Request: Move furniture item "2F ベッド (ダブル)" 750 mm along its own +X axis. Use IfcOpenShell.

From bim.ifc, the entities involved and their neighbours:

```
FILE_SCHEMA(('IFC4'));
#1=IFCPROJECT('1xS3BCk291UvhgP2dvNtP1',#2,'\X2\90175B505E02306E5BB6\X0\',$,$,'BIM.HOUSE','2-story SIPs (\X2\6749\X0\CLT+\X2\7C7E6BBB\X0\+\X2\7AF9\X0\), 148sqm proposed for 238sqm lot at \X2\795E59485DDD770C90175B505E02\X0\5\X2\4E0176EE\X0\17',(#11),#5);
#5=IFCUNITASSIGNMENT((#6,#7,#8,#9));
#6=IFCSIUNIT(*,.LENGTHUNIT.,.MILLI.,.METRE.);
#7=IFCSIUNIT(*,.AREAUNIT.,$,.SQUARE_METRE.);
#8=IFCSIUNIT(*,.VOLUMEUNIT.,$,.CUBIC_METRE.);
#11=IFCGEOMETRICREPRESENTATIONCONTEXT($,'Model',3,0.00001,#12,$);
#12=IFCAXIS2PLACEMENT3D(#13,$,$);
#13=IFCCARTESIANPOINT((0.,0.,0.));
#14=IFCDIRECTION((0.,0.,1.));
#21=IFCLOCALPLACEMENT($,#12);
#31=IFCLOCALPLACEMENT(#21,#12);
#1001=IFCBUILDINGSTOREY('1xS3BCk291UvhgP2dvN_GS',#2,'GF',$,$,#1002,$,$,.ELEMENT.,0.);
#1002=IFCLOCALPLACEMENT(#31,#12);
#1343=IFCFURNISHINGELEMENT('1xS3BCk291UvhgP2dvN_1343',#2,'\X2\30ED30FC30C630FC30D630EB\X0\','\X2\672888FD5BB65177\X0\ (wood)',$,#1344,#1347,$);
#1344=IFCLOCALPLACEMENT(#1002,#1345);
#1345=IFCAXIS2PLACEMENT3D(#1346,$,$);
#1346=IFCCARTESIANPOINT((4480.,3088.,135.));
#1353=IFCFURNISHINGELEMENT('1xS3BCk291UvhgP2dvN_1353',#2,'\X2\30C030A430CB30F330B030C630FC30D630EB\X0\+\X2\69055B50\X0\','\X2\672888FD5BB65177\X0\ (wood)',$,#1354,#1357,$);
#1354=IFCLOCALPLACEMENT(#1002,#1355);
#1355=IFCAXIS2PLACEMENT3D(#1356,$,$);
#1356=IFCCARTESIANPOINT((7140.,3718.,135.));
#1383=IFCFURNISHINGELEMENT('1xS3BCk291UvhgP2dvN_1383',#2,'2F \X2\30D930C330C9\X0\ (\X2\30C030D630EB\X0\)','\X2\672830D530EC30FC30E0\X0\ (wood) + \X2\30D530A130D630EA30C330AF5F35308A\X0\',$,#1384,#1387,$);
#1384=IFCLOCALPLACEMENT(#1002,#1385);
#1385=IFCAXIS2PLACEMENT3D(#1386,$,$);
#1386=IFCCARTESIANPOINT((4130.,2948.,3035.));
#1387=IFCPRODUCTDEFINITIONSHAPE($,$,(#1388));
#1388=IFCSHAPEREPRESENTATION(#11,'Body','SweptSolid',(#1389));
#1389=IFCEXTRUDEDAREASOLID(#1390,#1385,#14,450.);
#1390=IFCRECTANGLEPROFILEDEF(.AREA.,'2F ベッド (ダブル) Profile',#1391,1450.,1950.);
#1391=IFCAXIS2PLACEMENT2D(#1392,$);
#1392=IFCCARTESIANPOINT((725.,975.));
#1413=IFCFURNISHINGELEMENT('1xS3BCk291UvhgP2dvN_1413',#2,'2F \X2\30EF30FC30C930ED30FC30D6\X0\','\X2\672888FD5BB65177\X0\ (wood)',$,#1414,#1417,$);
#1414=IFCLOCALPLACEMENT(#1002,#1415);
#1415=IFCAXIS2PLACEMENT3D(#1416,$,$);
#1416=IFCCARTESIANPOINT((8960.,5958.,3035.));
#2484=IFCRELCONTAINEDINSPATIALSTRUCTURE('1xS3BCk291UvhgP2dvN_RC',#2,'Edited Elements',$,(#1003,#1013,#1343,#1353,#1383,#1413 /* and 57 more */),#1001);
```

```python
import ifcopenshell
import ifcopenshell.api.geometry
import ifcopenshell.util.placement
import ifcopenshell.util.unit

model = ifcopenshell.open("bim.ifc")
unit_scale = ifcopenshell.util.unit.calculate_unit_scale(model)

item = model.by_guid("1xS3BCk291UvhgP2dvN_1383")
matrix = ifcopenshell.util.placement.get_local_placement(item.ObjectPlacement)
matrix[:3, 3] += matrix[:3, 0] * 0.75 / unit_scale
ifcopenshell.api.geometry.edit_object_placement(model, product=item, matrix=matrix, is_si=False)

print(ifcopenshell.util.placement.get_local_placement(item.ObjectPlacement).round(3) + 0.0)

model.write("bim_rev.ifc")
```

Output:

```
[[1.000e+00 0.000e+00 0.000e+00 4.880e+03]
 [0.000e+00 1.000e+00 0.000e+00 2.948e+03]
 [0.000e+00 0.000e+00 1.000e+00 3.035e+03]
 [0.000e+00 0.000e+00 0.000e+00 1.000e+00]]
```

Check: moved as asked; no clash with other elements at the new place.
